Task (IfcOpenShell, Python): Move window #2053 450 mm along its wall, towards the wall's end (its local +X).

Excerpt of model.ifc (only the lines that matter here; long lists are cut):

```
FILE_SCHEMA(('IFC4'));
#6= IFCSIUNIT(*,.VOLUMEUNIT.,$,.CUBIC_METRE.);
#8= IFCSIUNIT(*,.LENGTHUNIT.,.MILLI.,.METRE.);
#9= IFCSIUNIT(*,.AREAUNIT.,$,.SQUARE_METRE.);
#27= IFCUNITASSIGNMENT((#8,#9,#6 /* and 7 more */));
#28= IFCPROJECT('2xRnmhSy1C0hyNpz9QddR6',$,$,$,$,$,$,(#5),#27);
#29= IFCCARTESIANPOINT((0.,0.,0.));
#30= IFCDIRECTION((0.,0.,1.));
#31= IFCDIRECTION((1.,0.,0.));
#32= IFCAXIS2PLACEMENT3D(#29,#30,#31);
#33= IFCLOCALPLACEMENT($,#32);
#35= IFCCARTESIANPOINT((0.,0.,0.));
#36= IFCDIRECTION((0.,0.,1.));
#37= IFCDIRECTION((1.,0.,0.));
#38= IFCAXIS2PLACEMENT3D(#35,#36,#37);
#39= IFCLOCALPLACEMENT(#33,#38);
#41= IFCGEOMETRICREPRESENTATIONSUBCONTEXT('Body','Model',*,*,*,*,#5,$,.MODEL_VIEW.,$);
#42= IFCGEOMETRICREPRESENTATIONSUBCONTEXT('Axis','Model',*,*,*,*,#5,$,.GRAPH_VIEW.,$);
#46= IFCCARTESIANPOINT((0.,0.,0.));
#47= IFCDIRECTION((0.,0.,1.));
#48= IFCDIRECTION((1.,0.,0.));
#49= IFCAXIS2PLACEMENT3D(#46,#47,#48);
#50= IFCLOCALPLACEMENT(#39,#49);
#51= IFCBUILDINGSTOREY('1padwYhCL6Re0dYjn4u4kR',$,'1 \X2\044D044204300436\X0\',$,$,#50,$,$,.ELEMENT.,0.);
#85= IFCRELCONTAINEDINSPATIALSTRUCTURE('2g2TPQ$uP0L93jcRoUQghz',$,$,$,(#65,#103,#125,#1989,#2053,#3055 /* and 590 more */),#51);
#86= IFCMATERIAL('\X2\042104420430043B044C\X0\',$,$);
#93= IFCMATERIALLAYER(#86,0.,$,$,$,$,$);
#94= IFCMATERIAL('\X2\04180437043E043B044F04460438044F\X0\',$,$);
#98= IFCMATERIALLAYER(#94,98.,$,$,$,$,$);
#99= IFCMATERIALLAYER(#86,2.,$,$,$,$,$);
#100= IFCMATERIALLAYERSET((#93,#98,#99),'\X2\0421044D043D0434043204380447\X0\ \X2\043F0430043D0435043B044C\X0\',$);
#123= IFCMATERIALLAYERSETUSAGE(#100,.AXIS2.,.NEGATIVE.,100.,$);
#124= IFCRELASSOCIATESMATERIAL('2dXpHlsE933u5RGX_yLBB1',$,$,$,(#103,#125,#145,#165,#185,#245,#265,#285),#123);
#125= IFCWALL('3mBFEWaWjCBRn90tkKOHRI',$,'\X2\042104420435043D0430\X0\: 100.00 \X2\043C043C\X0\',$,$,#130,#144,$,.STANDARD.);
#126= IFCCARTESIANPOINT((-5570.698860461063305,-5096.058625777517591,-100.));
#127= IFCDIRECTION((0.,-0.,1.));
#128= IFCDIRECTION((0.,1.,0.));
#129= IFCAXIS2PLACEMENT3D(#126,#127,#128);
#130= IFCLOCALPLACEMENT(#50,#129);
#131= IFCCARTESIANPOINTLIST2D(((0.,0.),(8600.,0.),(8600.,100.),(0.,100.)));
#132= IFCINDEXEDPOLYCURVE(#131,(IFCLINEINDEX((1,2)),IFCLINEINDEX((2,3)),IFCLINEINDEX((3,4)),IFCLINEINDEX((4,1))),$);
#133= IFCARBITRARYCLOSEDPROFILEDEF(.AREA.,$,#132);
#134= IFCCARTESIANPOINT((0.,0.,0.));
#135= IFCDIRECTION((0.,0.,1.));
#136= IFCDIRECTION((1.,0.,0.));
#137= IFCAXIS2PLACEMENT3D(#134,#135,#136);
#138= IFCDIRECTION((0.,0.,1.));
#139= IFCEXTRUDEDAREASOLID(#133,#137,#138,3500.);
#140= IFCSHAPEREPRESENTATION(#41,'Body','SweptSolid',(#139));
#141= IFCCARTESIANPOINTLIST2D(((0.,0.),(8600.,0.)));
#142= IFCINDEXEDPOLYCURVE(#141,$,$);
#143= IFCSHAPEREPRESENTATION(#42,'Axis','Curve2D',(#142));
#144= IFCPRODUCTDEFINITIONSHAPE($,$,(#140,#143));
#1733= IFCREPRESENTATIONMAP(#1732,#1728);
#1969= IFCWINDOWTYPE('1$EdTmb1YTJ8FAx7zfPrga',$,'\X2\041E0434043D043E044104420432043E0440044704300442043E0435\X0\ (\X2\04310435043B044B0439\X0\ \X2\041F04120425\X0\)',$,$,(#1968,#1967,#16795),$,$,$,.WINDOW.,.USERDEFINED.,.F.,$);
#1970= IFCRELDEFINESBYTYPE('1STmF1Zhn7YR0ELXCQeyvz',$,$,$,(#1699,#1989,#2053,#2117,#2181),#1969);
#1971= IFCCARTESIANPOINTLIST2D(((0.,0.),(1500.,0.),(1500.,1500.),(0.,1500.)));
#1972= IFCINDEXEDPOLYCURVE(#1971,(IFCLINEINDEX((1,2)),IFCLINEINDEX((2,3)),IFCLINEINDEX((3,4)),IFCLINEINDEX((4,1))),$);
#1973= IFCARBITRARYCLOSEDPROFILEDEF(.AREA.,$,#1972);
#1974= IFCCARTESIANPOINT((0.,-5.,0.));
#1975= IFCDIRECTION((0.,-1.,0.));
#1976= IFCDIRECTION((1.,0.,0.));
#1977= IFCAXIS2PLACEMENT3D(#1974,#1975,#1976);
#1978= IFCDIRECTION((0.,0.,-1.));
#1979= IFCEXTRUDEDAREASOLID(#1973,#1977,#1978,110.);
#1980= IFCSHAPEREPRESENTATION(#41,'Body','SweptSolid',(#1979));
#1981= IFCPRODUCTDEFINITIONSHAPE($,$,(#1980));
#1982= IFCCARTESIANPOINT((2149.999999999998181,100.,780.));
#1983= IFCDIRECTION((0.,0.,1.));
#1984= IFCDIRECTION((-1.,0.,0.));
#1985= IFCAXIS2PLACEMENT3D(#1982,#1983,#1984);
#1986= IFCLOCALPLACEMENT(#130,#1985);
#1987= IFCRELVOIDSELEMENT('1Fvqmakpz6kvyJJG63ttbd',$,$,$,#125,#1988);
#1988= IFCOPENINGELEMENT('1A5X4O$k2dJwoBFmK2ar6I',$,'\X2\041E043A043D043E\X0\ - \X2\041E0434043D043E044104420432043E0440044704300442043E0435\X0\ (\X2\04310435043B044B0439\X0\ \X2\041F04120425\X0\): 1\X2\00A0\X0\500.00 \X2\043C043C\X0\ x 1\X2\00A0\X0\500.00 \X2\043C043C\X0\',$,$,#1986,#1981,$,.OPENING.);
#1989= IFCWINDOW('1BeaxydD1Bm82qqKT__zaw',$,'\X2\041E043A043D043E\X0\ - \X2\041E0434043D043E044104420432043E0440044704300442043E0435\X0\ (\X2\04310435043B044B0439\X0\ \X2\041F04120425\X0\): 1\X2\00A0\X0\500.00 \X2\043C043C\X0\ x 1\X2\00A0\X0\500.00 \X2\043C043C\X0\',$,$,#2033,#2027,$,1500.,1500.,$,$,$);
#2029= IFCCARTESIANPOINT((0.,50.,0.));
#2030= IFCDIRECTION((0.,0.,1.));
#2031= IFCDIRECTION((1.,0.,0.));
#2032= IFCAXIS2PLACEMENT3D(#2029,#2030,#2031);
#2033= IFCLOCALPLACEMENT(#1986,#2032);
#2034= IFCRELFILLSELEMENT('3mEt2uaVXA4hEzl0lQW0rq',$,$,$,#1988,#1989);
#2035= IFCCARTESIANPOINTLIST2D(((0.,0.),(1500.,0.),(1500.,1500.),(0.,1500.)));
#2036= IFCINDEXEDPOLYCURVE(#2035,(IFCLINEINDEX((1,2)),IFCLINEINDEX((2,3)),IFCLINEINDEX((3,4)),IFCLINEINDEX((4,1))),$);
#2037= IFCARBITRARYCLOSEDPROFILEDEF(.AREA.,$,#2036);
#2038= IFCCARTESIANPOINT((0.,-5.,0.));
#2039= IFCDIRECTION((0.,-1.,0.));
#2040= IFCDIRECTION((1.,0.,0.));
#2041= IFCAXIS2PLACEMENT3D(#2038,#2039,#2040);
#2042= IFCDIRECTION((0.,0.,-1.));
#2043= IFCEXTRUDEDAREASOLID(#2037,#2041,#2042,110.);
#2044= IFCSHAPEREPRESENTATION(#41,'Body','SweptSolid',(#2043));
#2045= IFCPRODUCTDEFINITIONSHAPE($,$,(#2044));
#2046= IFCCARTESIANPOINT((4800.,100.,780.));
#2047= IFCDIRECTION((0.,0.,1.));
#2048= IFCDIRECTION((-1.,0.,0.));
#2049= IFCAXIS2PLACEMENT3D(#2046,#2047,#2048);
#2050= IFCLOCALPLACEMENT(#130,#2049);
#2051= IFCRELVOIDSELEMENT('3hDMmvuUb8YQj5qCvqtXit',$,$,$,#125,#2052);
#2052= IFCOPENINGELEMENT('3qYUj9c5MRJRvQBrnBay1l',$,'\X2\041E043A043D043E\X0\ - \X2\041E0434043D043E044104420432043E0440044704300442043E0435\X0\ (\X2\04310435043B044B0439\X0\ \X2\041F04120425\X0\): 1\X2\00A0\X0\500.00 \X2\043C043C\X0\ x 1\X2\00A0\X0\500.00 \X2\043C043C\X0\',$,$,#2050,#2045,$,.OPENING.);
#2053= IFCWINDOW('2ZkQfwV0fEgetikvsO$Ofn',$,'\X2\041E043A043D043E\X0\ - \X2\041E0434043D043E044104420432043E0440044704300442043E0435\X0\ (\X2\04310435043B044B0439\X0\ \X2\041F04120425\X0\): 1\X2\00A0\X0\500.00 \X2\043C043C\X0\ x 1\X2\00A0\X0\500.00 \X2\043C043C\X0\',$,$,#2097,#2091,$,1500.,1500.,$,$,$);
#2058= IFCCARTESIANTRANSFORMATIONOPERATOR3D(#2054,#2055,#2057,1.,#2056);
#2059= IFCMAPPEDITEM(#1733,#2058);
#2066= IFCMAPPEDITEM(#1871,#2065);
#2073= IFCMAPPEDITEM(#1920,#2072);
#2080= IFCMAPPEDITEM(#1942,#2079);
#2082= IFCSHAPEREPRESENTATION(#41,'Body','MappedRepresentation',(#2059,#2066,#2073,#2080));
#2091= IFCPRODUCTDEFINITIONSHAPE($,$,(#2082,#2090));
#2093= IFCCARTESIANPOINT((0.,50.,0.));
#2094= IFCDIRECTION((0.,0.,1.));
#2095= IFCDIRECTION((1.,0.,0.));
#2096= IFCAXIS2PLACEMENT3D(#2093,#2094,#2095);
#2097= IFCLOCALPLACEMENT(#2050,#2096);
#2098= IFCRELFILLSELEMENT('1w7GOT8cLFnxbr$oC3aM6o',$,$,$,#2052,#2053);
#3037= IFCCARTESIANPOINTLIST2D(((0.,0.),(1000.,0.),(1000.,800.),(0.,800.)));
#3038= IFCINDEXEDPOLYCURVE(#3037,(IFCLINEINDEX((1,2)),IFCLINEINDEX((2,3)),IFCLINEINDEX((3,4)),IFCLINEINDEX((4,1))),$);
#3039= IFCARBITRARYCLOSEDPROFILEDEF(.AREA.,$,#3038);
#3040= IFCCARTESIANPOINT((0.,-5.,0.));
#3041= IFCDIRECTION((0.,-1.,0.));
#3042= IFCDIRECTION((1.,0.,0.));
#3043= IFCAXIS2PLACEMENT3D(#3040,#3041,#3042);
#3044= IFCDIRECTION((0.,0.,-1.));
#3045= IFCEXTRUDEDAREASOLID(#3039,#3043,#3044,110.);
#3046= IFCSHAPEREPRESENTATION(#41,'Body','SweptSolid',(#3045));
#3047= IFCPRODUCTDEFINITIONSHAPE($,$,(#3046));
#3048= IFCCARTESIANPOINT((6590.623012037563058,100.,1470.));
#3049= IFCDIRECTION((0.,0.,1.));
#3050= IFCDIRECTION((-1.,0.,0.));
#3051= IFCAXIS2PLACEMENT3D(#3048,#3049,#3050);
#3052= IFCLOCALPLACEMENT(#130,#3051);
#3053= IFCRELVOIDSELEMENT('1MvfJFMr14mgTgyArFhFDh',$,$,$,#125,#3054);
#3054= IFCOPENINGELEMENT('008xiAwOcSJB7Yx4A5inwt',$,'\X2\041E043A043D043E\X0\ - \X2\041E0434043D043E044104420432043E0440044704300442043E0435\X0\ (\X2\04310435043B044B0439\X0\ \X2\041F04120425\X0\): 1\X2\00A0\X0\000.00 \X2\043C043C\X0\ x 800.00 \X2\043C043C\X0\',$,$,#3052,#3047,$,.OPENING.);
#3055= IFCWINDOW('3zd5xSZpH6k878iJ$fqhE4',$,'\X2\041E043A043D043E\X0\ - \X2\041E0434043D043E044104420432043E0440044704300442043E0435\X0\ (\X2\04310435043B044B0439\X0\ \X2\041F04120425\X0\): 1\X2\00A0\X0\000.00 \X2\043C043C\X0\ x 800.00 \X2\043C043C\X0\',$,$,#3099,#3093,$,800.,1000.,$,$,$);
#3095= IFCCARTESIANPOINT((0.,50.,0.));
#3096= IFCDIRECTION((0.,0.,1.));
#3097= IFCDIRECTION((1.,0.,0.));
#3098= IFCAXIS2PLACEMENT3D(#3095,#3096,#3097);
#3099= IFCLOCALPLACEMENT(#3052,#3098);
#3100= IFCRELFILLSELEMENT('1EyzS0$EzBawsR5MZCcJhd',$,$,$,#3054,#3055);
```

```python
import ifcopenshell
import ifcopenshell.api.geometry
import ifcopenshell.util.placement

model = ifcopenshell.open("model.ifc")

window = model.by_id(2053)
opening = window.FillsVoids[0].RelatingOpeningElement
wall = opening.VoidsElements[0].RelatingBuildingElement

wall_matrix = ifcopenshell.util.placement.get_local_placement(wall.ObjectPlacement)
shift = wall_matrix[:3, 0] * 450.0
before = ifcopenshell.util.placement.get_local_placement(window.ObjectPlacement)[:3, 3].copy()

# The window is placed relative to its opening, so it follows when the opening moves.
matrix = ifcopenshell.util.placement.get_local_placement(opening.ObjectPlacement)
matrix[:3, 3] += shift
ifcopenshell.api.geometry.edit_object_placement(
    model, product=opening, matrix=matrix, is_si=False, should_transform_children=True
)

after = ifcopenshell.util.placement.get_local_placement(window.ObjectPlacement)[:3, 3]
print("window moved by", (after - before).round(3) + 0.0)

model.write("model_edited.ifc")
```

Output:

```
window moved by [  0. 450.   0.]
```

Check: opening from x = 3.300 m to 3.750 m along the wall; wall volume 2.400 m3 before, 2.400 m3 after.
